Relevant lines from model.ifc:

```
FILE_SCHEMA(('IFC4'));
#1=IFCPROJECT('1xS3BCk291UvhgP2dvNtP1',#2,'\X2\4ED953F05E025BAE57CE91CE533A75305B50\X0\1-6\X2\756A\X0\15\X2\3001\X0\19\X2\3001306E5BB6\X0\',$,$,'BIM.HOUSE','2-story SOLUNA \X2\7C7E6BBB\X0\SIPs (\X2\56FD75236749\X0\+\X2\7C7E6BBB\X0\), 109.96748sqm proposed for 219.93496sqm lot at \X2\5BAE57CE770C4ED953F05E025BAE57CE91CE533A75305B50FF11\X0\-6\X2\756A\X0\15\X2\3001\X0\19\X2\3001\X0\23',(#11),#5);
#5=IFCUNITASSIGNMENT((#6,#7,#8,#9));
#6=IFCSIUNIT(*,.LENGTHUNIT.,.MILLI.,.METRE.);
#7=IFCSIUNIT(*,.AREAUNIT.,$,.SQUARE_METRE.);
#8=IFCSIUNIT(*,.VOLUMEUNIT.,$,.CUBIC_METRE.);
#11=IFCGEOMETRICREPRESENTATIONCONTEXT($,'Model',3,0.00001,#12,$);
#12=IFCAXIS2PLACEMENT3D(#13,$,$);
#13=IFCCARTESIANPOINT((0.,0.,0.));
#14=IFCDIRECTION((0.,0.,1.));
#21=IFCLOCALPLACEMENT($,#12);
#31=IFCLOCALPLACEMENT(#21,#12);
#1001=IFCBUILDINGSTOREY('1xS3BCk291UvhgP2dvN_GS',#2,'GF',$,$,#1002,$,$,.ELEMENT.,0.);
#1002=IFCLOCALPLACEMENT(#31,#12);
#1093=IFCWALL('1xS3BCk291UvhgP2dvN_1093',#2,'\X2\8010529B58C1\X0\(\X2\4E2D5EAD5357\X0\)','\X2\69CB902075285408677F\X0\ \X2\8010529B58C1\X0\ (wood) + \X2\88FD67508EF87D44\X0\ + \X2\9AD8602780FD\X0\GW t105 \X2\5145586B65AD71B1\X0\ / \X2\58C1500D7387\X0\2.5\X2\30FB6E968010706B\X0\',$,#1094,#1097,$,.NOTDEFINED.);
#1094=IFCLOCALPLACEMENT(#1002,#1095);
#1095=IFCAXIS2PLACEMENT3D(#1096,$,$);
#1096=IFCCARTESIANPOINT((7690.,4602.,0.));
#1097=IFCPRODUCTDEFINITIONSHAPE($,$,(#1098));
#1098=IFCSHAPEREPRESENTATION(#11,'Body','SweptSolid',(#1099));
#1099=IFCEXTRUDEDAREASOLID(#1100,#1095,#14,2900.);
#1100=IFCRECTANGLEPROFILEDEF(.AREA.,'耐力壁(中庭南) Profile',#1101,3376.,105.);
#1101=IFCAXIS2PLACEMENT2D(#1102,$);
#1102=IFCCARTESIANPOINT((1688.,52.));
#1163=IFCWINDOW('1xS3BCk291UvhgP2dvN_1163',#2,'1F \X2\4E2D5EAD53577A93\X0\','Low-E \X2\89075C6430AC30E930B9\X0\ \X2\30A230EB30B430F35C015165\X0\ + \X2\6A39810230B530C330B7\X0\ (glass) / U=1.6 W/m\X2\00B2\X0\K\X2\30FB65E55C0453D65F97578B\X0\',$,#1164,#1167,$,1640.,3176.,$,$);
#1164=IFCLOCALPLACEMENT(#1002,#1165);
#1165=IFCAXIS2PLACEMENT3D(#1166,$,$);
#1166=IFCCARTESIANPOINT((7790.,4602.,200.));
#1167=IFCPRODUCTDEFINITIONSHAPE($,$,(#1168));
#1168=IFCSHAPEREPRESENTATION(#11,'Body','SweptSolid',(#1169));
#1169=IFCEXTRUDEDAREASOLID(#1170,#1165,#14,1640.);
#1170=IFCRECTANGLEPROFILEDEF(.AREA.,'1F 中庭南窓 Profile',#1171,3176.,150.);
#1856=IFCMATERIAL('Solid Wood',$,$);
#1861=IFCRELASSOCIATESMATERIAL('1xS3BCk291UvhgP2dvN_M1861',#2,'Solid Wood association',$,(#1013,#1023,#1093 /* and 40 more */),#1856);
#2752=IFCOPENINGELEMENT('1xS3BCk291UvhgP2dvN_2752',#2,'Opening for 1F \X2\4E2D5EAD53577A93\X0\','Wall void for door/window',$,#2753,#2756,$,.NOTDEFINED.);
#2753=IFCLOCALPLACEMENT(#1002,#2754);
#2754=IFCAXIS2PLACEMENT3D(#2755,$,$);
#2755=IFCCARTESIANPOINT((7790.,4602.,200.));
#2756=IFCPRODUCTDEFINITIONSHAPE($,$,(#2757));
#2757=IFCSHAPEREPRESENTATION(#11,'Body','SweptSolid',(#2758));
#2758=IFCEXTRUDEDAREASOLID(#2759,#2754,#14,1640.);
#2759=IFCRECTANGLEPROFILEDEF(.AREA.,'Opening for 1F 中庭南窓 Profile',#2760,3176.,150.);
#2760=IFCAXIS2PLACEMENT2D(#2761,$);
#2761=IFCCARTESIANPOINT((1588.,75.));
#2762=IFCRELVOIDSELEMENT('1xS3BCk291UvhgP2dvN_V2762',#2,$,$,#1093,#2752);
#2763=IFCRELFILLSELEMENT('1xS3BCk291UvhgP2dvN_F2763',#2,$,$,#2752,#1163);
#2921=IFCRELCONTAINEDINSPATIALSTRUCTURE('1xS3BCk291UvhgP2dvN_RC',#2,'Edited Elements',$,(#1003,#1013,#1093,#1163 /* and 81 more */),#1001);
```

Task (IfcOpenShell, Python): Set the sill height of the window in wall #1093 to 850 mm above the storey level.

```python
import numpy as np
import ifcopenshell
import ifcopenshell.api.geometry
import ifcopenshell.geom
import ifcopenshell.util.element
import ifcopenshell.util.placement
import ifcopenshell.util.shape
import ifcopenshell.util.unit

model = ifcopenshell.open("model.ifc")
unit_scale = ifcopenshell.util.unit.calculate_unit_scale(model)

window = model.by_guid("1xS3BCk291UvhgP2dvN_1163")
opening = window.FillsVoids[0].RelatingOpeningElement
storey = ifcopenshell.util.element.get_container(window, ifc_class="IfcBuildingStorey")
level = ifcopenshell.util.placement.get_local_placement(storey.ObjectPlacement)[2, 3]

# The opening's origin need not be at the sill, so measure its lowest point.
shape = ifcopenshell.geom.create_shape(ifcopenshell.geom.settings(), opening)
bottom = ifcopenshell.util.shape.get_shape_bottom_elevation(shape, shape.geometry) / unit_scale
dz = level + 850.0 - bottom

shift = np.array([0.0, 0.0, dz])
# The window is not placed relative to its opening, so move both.
for product in (opening, window):
    matrix = ifcopenshell.util.placement.get_local_placement(product.ObjectPlacement)
    matrix[:3, 3] += shift
    ifcopenshell.api.geometry.edit_object_placement(model, product=product, matrix=matrix, is_si=False)

print(f"moved by {dz * unit_scale:+.3f} m")

model.write("model_rev.ifc")
```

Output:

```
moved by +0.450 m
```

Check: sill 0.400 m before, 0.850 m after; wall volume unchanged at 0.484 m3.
